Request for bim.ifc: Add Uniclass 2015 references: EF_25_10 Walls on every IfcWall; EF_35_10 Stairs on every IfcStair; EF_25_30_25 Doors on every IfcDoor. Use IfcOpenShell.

First a look at what the model holds.

```python
import ifcopenshell

model = ifcopenshell.open("bim.ifc")
print(model.schema)
print("classifications:", [c.Name for c in model.by_type("IfcClassification")])
for ifc_class in ("IfcDoor", "IfcRoof", "IfcStair", "IfcWall", "IfcWindow"):
    print(ifc_class, len(model.by_type(ifc_class)))
```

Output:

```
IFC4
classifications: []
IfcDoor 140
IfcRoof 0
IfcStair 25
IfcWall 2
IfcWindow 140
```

```python
import ifcopenshell
import ifcopenshell.api.classification

model = ifcopenshell.open("bim.ifc")

system = ifcopenshell.api.classification.add_classification(model, classification="Uniclass 2015")

codes = {
    "IfcWall": ("EF_25_10", "Walls"),
    "IfcStair": ("EF_35_10", "Stairs"),
    "IfcDoor": ("EF_25_30_25", "Doors"),
}
for ifc_class, (code, name) in codes.items():
    products = model.by_type(ifc_class)
    ifcopenshell.api.classification.add_reference(
        model, products=products, classification=system, identification=code, name=name
    )
    print(code, len(products))

model.write("bim_v2.ifc")
```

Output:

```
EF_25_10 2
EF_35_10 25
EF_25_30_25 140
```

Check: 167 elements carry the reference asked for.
